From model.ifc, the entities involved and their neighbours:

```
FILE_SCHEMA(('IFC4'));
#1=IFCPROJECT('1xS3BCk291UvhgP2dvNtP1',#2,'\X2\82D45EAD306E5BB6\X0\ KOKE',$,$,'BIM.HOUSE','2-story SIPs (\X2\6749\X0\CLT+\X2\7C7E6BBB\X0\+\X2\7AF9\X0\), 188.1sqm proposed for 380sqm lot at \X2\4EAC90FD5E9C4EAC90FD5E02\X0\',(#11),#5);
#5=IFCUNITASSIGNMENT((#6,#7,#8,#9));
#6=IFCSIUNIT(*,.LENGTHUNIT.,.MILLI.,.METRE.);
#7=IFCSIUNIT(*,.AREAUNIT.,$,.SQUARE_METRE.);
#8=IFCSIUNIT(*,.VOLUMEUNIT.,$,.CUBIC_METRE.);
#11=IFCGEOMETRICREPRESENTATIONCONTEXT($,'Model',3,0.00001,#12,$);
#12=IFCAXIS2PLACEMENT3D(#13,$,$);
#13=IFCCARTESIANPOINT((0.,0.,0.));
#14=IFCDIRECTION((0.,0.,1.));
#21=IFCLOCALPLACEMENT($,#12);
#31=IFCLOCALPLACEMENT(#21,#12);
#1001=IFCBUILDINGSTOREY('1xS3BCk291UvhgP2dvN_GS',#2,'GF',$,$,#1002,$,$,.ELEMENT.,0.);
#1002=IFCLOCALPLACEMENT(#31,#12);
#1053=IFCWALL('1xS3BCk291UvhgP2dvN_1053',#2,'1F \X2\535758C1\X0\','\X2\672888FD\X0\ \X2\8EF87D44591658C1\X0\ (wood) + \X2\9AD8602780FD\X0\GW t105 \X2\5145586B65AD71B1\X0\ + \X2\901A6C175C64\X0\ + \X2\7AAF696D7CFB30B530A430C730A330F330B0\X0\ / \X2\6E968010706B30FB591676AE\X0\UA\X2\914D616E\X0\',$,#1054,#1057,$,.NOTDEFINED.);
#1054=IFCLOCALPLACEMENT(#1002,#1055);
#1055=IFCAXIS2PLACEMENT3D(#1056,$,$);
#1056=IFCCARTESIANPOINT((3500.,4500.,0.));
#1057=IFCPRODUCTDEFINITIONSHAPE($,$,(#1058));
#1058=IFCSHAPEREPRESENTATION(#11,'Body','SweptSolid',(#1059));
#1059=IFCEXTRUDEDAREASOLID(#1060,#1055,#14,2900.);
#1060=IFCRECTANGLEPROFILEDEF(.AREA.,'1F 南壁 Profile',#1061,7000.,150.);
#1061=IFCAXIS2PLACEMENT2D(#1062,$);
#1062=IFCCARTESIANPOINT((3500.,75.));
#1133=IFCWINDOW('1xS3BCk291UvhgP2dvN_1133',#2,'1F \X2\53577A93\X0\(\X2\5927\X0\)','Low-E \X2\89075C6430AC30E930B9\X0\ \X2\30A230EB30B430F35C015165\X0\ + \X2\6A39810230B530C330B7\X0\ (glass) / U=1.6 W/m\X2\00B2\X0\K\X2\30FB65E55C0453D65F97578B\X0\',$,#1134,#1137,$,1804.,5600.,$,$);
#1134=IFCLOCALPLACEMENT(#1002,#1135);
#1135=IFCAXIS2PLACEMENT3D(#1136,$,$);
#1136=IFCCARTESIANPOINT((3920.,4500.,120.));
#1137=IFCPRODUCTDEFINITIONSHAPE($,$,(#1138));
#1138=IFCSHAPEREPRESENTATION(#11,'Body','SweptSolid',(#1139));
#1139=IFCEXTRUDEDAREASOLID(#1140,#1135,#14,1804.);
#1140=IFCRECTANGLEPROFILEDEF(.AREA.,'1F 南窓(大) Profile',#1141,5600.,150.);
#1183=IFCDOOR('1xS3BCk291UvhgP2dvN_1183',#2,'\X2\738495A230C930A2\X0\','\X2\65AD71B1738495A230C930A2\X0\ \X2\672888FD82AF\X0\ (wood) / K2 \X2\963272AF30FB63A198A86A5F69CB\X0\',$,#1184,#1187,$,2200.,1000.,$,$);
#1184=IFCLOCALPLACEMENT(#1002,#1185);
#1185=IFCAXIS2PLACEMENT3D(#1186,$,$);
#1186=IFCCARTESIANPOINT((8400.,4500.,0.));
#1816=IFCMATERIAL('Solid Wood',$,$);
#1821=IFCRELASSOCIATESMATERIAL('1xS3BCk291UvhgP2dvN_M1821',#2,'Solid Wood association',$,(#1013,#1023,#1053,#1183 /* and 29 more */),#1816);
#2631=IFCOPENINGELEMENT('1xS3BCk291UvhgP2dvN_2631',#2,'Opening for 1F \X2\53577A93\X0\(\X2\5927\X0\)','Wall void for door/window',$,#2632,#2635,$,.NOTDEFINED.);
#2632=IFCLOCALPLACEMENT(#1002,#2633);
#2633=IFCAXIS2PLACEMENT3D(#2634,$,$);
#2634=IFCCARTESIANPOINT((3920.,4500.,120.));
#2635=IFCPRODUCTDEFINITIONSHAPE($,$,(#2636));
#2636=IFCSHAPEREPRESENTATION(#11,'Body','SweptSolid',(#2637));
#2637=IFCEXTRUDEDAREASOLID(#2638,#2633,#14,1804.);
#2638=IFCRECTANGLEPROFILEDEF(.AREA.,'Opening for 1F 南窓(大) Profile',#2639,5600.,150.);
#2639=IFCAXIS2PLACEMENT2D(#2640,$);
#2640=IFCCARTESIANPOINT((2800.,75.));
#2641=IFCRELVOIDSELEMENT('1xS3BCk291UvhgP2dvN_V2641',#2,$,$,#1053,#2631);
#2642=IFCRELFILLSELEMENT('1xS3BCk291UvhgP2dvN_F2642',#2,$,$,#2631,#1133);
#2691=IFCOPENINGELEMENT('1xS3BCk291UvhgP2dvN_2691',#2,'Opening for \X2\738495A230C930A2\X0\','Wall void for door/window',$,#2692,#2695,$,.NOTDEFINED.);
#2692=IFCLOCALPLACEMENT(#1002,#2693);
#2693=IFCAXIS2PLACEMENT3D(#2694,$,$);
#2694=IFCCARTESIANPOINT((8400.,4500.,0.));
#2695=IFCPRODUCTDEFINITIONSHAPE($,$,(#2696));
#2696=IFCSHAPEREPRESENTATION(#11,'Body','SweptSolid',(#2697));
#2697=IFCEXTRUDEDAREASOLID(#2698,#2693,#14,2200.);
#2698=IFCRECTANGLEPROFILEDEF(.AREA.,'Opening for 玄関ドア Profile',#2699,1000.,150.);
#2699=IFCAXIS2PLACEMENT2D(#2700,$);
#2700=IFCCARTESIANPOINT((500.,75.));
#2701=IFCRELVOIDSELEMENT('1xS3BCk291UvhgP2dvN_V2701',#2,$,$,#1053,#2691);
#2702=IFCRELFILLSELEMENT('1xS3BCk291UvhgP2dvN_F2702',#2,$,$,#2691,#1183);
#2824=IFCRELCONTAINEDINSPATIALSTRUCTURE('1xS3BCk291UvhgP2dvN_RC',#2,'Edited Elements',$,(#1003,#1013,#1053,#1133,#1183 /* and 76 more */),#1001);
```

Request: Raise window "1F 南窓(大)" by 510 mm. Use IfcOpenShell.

```python
import numpy as np
import ifcopenshell
import ifcopenshell.api.geometry
import ifcopenshell.util.placement
import ifcopenshell.util.unit

model = ifcopenshell.open("model.ifc")
unit_scale = ifcopenshell.util.unit.calculate_unit_scale(model)

window = model.by_guid("1xS3BCk291UvhgP2dvN_1133")
opening = window.FillsVoids[0].RelatingOpeningElement
dz = 0.51 / unit_scale

shift = np.array([0.0, 0.0, dz])
# The window is not placed relative to its opening, so move both.
for product in (opening, window):
    matrix = ifcopenshell.util.placement.get_local_placement(product.ObjectPlacement)
    matrix[:3, 3] += shift
    ifcopenshell.api.geometry.edit_object_placement(model, product=product, matrix=matrix, is_si=False)

print(f"moved by {dz * unit_scale:+.3f} m")

model.write("model-out.ifc")
```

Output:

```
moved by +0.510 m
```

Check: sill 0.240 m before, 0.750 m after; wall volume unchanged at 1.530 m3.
